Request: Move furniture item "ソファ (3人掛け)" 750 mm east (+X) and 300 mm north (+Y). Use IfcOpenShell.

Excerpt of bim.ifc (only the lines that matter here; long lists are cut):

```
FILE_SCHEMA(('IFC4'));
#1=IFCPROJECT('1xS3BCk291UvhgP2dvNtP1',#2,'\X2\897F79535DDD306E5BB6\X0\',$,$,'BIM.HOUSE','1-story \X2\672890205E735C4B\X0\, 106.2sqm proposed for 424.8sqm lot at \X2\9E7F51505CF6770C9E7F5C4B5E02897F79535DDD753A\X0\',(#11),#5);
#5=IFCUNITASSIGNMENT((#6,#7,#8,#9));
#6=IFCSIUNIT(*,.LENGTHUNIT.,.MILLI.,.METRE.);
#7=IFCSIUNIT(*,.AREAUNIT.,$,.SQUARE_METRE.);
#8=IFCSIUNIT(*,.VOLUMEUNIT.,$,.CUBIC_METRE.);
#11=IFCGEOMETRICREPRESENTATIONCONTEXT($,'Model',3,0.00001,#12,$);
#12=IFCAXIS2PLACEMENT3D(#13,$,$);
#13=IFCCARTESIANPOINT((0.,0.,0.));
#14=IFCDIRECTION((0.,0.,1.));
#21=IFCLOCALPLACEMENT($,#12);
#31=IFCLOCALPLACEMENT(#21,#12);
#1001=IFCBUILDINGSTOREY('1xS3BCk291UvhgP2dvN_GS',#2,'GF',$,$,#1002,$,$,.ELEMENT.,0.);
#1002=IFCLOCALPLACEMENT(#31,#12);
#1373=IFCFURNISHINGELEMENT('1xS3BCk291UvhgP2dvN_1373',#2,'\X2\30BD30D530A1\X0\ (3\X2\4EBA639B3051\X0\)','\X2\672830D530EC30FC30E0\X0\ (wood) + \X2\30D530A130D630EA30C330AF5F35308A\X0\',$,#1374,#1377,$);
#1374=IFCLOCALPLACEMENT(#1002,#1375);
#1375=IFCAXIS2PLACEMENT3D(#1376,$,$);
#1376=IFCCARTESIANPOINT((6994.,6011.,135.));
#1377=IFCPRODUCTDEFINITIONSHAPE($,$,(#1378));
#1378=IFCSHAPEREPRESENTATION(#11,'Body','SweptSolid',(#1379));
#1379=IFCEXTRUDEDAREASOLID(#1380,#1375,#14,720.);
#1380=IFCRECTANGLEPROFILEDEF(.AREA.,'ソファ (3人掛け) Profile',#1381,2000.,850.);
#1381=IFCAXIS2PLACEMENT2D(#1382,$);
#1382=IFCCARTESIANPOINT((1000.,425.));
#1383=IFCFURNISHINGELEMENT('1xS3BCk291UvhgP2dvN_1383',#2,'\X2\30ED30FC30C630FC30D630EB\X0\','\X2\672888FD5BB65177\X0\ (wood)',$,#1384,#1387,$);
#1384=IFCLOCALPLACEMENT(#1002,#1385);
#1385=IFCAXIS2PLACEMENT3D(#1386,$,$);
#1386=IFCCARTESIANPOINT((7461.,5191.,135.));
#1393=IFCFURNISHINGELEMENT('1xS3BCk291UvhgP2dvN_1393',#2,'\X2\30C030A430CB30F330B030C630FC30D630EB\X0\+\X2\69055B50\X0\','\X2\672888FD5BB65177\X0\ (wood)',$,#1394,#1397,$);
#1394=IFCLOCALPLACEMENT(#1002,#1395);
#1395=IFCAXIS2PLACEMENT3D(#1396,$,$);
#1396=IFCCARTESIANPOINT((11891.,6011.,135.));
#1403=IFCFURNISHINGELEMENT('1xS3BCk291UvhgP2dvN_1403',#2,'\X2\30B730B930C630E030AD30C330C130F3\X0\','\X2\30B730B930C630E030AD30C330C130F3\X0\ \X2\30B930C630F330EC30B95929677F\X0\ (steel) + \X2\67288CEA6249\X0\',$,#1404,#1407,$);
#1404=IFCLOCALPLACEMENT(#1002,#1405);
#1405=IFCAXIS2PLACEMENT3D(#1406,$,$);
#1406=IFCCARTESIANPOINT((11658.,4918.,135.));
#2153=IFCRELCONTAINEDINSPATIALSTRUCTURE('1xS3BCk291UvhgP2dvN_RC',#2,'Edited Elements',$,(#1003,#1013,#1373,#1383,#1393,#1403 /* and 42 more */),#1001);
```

```python
import ifcopenshell
import ifcopenshell.api.geometry
import ifcopenshell.util.placement

model = ifcopenshell.open("bim.ifc")

item = model.by_id(1373)
matrix = ifcopenshell.util.placement.get_local_placement(item.ObjectPlacement)
matrix[0, 3] += 750.0
matrix[1, 3] += 300.0
ifcopenshell.api.geometry.edit_object_placement(model, product=item, matrix=matrix, is_si=False)

print(ifcopenshell.util.placement.get_local_placement(item.ObjectPlacement).round(3) + 0.0)

model.write("bim-out.ifc")
```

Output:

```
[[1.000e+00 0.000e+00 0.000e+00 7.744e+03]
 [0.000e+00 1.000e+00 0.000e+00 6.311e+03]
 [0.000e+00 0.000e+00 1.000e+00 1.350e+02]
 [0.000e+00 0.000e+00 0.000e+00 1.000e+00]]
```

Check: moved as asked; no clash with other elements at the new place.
